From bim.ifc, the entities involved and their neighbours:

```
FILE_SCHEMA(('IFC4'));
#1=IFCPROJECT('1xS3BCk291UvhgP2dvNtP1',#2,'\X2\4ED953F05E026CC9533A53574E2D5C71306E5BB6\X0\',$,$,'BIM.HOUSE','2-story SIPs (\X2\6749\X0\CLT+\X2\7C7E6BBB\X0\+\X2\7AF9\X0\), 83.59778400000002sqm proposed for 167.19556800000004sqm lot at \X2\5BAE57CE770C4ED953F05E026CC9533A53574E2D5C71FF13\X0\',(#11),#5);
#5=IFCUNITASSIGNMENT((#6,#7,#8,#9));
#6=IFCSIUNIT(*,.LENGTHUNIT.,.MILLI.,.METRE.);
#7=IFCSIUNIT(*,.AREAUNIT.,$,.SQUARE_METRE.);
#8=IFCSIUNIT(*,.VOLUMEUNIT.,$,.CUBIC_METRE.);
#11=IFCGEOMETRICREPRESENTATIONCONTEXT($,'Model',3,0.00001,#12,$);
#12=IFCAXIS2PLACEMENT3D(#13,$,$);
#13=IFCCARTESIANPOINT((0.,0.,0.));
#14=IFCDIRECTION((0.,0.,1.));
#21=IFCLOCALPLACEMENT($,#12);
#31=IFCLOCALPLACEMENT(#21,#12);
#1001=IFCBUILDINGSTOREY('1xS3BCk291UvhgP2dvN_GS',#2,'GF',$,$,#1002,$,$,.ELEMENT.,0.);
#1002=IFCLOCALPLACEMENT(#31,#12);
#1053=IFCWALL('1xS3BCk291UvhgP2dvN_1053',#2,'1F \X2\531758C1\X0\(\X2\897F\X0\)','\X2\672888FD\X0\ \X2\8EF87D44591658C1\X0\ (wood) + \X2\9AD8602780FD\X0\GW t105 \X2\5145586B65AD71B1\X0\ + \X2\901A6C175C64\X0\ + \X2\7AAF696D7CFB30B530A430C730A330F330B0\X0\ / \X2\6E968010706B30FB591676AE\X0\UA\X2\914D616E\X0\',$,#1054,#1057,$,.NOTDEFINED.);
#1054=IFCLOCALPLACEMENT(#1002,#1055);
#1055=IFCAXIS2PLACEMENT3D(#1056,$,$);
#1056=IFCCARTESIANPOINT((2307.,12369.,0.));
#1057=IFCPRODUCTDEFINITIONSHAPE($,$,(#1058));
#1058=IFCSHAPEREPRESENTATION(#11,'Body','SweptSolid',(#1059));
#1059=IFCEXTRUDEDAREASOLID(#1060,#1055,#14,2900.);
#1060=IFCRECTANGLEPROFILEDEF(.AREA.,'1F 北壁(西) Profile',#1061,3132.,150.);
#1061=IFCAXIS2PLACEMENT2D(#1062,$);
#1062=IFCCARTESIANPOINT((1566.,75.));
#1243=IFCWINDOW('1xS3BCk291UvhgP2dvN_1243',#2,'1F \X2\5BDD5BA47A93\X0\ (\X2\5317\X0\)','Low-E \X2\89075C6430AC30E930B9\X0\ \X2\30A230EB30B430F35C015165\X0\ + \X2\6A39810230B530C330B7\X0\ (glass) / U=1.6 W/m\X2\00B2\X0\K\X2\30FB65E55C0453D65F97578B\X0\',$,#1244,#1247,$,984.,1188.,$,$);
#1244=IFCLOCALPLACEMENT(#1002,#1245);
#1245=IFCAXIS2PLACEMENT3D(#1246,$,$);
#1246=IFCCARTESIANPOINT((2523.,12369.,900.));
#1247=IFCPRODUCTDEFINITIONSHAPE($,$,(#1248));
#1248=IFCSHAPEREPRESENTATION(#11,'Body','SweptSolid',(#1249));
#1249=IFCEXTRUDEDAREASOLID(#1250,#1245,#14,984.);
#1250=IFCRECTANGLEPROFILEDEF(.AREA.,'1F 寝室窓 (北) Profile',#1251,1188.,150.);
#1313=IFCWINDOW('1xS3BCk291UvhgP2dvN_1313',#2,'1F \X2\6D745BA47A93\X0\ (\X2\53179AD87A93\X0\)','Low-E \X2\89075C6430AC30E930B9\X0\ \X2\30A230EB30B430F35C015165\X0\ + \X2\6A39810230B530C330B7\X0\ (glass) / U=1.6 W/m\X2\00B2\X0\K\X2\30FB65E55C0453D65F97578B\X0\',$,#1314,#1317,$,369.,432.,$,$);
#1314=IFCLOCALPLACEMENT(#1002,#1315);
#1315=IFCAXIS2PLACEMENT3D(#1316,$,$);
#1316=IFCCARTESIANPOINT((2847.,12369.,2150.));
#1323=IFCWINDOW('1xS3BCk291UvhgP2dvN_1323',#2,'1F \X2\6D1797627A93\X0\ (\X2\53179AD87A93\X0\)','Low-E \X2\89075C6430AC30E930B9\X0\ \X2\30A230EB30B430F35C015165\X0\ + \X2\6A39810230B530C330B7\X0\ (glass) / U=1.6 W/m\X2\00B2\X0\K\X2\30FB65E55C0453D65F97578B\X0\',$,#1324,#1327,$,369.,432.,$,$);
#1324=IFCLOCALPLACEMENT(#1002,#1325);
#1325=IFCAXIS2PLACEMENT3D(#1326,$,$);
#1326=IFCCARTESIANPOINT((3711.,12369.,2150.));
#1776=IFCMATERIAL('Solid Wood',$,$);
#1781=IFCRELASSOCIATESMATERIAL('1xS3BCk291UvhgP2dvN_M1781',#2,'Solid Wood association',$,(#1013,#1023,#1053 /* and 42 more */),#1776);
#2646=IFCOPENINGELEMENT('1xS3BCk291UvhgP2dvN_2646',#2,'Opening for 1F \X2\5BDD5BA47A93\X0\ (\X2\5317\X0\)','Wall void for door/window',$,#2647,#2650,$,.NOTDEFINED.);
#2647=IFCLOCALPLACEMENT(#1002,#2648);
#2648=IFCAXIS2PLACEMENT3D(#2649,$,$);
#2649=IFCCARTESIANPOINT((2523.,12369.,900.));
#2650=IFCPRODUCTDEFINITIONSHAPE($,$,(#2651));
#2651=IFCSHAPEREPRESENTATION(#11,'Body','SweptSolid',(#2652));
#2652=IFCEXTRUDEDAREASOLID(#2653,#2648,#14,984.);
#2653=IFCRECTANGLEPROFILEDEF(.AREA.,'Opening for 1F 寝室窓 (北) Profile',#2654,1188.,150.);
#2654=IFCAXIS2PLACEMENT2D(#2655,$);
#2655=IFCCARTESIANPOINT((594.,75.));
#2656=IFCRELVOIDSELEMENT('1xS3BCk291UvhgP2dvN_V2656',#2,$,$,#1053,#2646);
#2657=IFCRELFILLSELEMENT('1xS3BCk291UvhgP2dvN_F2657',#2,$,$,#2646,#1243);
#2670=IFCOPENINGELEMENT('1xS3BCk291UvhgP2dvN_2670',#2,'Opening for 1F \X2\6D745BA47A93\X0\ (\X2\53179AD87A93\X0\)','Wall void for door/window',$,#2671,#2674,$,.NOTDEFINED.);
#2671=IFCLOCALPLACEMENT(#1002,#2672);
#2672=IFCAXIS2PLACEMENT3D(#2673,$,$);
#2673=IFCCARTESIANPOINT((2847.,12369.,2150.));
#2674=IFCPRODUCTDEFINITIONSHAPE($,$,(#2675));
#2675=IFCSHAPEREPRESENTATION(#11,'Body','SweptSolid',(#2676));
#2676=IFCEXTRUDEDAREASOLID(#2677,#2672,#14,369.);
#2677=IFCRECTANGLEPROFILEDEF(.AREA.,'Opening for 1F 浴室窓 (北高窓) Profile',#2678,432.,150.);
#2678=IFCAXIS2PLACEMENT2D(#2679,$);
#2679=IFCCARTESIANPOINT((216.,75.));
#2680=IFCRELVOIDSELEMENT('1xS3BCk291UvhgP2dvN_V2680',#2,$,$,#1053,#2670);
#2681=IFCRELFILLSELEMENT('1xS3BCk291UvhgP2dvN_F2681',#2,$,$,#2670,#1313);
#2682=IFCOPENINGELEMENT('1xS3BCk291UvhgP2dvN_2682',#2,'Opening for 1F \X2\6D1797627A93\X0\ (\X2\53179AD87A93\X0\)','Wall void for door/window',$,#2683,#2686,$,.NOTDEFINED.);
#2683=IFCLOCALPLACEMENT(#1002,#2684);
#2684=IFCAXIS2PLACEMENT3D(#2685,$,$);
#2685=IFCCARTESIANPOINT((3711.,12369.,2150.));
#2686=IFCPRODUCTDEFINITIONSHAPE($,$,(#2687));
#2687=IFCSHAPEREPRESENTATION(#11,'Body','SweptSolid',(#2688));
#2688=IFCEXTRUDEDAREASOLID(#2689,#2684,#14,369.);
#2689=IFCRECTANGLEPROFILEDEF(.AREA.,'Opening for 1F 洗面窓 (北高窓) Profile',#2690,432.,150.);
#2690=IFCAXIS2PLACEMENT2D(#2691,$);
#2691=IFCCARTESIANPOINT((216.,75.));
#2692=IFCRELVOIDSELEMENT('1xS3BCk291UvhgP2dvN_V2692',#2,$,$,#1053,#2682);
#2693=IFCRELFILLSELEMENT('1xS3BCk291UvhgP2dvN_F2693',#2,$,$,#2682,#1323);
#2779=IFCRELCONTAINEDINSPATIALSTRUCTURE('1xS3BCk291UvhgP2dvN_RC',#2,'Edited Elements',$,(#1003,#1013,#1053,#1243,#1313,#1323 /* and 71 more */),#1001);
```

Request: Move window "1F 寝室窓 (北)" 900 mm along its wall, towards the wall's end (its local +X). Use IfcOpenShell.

```python
import ifcopenshell
import ifcopenshell.api.geometry
import ifcopenshell.util.placement

model = ifcopenshell.open("bim.ifc")

window = model.by_id(1243)
opening = window.FillsVoids[0].RelatingOpeningElement
wall = opening.VoidsElements[0].RelatingBuildingElement

wall_matrix = ifcopenshell.util.placement.get_local_placement(wall.ObjectPlacement)
shift = wall_matrix[:3, 0] * 900.0
before = ifcopenshell.util.placement.get_local_placement(window.ObjectPlacement)[:3, 3].copy()

# The window is not placed relative to its opening, so move both.
for product in (opening, window):
    matrix = ifcopenshell.util.placement.get_local_placement(product.ObjectPlacement)
    matrix[:3, 3] += shift
    ifcopenshell.api.geometry.edit_object_placement(model, product=product, matrix=matrix, is_si=False)

after = ifcopenshell.util.placement.get_local_placement(window.ObjectPlacement)[:3, 3]
print("window moved by", (after - before).round(3) + 0.0)

model.write("bim-out.ifc")
```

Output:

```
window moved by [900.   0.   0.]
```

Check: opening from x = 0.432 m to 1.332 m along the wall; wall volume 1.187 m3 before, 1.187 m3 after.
